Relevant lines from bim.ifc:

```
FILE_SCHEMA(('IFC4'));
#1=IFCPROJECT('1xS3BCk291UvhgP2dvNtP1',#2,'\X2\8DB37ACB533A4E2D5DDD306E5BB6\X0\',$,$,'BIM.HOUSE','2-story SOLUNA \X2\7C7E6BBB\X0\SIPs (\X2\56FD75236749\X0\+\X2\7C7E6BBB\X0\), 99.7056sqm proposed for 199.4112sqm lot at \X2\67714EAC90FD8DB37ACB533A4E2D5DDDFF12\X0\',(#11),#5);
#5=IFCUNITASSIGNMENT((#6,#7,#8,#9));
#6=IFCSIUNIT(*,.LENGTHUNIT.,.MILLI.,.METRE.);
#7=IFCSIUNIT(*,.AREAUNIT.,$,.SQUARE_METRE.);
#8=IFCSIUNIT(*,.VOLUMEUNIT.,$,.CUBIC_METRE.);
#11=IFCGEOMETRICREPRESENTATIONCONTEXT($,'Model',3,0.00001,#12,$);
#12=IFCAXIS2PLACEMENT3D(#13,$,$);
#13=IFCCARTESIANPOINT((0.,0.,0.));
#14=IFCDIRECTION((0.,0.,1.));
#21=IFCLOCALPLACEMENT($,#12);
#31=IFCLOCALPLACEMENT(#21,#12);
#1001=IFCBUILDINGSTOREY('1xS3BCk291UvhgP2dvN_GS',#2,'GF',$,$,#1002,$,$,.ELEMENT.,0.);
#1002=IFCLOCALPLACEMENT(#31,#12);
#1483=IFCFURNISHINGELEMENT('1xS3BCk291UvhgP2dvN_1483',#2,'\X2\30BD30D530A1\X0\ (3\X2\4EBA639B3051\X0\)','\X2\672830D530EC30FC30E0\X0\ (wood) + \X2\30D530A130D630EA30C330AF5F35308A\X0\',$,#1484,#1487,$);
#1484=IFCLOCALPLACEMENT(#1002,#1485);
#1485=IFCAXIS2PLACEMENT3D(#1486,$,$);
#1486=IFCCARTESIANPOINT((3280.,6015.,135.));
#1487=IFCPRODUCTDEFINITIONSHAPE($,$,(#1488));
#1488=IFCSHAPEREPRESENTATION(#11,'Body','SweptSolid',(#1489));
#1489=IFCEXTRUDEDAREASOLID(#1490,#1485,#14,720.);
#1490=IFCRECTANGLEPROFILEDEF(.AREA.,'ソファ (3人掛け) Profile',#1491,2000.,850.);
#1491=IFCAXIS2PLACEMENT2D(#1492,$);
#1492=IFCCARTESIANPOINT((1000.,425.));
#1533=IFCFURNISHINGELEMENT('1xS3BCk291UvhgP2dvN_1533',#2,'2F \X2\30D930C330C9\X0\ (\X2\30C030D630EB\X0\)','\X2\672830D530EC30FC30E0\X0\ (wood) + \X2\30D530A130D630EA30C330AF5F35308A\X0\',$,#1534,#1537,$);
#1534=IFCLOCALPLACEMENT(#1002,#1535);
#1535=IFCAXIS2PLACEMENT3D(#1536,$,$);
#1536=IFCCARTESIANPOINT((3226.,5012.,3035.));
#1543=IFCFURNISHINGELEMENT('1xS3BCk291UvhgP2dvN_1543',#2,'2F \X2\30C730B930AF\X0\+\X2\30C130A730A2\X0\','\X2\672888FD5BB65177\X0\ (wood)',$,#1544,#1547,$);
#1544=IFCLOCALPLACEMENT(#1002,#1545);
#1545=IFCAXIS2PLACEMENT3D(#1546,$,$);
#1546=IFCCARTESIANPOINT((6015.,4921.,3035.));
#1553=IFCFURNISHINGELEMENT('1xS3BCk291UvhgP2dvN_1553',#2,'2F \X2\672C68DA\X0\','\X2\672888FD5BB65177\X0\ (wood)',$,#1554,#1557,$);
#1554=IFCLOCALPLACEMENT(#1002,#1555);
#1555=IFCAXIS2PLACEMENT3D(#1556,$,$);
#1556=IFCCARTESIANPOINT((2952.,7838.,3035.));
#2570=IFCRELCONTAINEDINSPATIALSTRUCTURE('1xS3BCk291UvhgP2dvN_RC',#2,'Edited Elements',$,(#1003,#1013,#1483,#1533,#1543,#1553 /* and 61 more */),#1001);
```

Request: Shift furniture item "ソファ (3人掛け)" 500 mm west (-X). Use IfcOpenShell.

```python
import ifcopenshell
import ifcopenshell.api.geometry
import ifcopenshell.util.placement
import ifcopenshell.util.unit

model = ifcopenshell.open("bim.ifc")
unit_scale = ifcopenshell.util.unit.calculate_unit_scale(model)

item = model.by_id(1483)
matrix = ifcopenshell.util.placement.get_local_placement(item.ObjectPlacement)
matrix[0, 3] -= 0.5 / unit_scale
ifcopenshell.api.geometry.edit_object_placement(model, product=item, matrix=matrix, is_si=False)

print(ifcopenshell.util.placement.get_local_placement(item.ObjectPlacement).round(3) + 0.0)

model.write("bim_rev.ifc")
```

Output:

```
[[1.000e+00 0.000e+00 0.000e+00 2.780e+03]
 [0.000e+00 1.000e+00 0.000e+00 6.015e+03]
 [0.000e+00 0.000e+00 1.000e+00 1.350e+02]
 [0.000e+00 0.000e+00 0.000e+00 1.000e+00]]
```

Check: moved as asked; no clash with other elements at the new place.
